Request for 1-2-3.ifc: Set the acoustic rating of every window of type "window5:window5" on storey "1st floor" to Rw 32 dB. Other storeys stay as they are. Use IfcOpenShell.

First a look at what the model holds.

```python
import ifcopenshell
import ifcopenshell.util.element

model = ifcopenshell.open("1-2-3.ifc")
print(model.schema)
storey = next(s for s in model.by_type("IfcBuildingStorey") if s.Name == "1st floor")
windows = [e for e in ifcopenshell.util.element.get_decomposition(storey) if e.is_a("IfcWindow")]
seen = {}
for e in windows:
    element_type = ifcopenshell.util.element.get_type(e)
    key = (element_type.Name if element_type != e and element_type else None, ifcopenshell.util.element.get_pset(e, "Pset_WindowCommon", "AcousticRating"))
    seen[key] = seen.get(key, 0) + 1
for (name, value), count in sorted(seen.items(), key=str):
    print(count, "x", name, "|", value)
```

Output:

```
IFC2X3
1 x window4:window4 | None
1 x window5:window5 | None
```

```python
import ifcopenshell
import ifcopenshell.api.pset
import ifcopenshell.util.element

model = ifcopenshell.open("1-2-3.ifc")

storey = next(s for s in model.by_type("IfcBuildingStorey") if s.Name == "1st floor")
windows = [e for e in ifcopenshell.util.element.get_decomposition(storey) if e.is_a("IfcWindow")]

count = 0
for e in windows:
    element_type = ifcopenshell.util.element.get_type(e)
    if element_type in (None, e) or element_type.Name != "window5:window5":
        continue
    # add_pset returns the element's existing set when there is one.
    pset = ifcopenshell.api.pset.add_pset(model, product=e, name="Pset_WindowCommon")
    ifcopenshell.api.pset.edit_pset(model, pset=pset, properties={"AcousticRating": "Rw 32 dB"})
    count += 1

print(count, "windows updated")

model.write("1-2-3_edited.ifc")
```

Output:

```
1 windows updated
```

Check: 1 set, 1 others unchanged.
